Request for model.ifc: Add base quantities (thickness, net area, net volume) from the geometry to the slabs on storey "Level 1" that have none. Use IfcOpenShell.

First a look at what the model holds.

```python
import ifcopenshell
import ifcopenshell.util.element
import ifcopenshell.util.unit

model = ifcopenshell.open("model.ifc")
print(model.schema)
for unit_type in ("LENGTHUNIT", "AREAUNIT", "VOLUMEUNIT"):
    print(unit_type, ifcopenshell.util.unit.calculate_unit_scale(model, unit_type))
storey = next(s for s in model.by_type("IfcBuildingStorey") if s.Name == "Level 1")
slabs = [e for e in ifcopenshell.util.element.get_decomposition(storey) if e.is_a("IfcSlab")]
for e in sorted(slabs, key=lambda e: e.id()):
    print(e.id(), e.is_a(), e.Name, list(ifcopenshell.util.element.get_psets(e, qtos_only=True)), sep=" | ")
```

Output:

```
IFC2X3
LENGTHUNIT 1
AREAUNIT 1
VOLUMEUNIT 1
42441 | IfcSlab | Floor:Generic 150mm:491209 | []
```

```python
import ifcopenshell
import ifcopenshell.api.pset
import ifcopenshell.geom
import ifcopenshell.util.element
import ifcopenshell.util.shape
import ifcopenshell.util.unit

model = ifcopenshell.open("model.ifc")
unit_scale = ifcopenshell.util.unit.calculate_unit_scale(model)
area_scale = ifcopenshell.util.unit.calculate_unit_scale(model, "AREAUNIT")
volume_scale = ifcopenshell.util.unit.calculate_unit_scale(model, "VOLUMEUNIT")
settings = ifcopenshell.geom.settings()

storey = next(s for s in model.by_type("IfcBuildingStorey") if s.Name == "Level 1")
slabs = [e for e in ifcopenshell.util.element.get_decomposition(storey) if e.is_a("IfcSlab")]

for e in sorted(slabs, key=lambda e: e.id()):
    if ifcopenshell.util.element.get_psets(e, qtos_only=True, should_inherit=False):
        continue
    # Geometry comes back in metres, in the element's own axes.
    shape = ifcopenshell.geom.create_shape(settings, e)
    values = {
        "Width": ifcopenshell.util.shape.get_z(shape.geometry) / unit_scale,
        "NetArea": ifcopenshell.util.shape.get_footprint_area(shape.geometry) / area_scale,
        "NetVolume": ifcopenshell.util.shape.get_volume(shape.geometry) / volume_scale,
    }
    qto = ifcopenshell.api.pset.add_qto(model, product=e, name="BaseQuantities")
    ifcopenshell.api.pset.edit_qto(model, qto=qto, properties=values)
    print(e.id(), {k: round(v, 3) for k, v in values.items()})

model.write("model_updated.ifc")
```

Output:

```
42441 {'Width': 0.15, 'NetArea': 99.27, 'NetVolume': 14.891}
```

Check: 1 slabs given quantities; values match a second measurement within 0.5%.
